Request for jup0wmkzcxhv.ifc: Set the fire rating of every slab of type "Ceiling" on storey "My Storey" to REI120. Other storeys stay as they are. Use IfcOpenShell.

First a look at what the model holds.

```python
import ifcopenshell
import ifcopenshell.util.element

model = ifcopenshell.open("jup0wmkzcxhv.ifc")
print(model.schema)
storey = next(s for s in model.by_type("IfcBuildingStorey") if s.Name == "My Storey")
slabs = [e for e in ifcopenshell.util.element.get_decomposition(storey) if e.is_a("IfcSlab")]
seen = {}
for e in slabs:
    element_type = ifcopenshell.util.element.get_type(e)
    key = (element_type.Name if element_type != e and element_type else None, ifcopenshell.util.element.get_pset(e, "Pset_SlabCommon", "FireRating"))
    seen[key] = seen.get(key, 0) + 1
for (name, value), count in sorted(seen.items(), key=str):
    print(count, "x", name, "|", value)
```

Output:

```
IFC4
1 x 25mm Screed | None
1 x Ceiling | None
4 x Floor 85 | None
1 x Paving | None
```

```python
import ifcopenshell
import ifcopenshell.api.pset
import ifcopenshell.util.element

model = ifcopenshell.open("jup0wmkzcxhv.ifc")

storey = next(s for s in model.by_type("IfcBuildingStorey") if s.Name == "My Storey")
slabs = [e for e in ifcopenshell.util.element.get_decomposition(storey) if e.is_a("IfcSlab")]

count = 0
for e in slabs:
    element_type = ifcopenshell.util.element.get_type(e)
    if element_type in (None, e) or element_type.Name != "Ceiling":
        continue
    # add_pset returns the element's existing set when there is one.
    pset = ifcopenshell.api.pset.add_pset(model, product=e, name="Pset_SlabCommon")
    ifcopenshell.api.pset.edit_pset(model, pset=pset, properties={"FireRating": "REI120"})
    count += 1

print(count, "slabs updated")

model.write("jup0wmkzcxhv-out.ifc")
```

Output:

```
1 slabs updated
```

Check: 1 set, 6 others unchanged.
